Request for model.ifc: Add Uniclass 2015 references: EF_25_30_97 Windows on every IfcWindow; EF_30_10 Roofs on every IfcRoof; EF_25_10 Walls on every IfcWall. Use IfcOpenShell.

First a look at what the model holds.

```python
import ifcopenshell

model = ifcopenshell.open("model.ifc")
print(model.schema)
print("classifications:", [c.Name for c in model.by_type("IfcClassification")])
for ifc_class in ("IfcDoor", "IfcRoof", "IfcStair", "IfcWall", "IfcWindow"):
    print(ifc_class, len(model.by_type(ifc_class)))
```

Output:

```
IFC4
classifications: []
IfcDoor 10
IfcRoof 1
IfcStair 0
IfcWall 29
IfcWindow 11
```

```python
import ifcopenshell
import ifcopenshell.api.classification

model = ifcopenshell.open("model.ifc")

system = ifcopenshell.api.classification.add_classification(model, classification="Uniclass 2015")

codes = {
    "IfcWindow": ("EF_25_30_97", "Windows"),
    "IfcRoof": ("EF_30_10", "Roofs"),
    "IfcWall": ("EF_25_10", "Walls"),
}
for ifc_class, (code, name) in codes.items():
    products = model.by_type(ifc_class)
    ifcopenshell.api.classification.add_reference(
        model, products=products, classification=system, identification=code, name=name
    )
    print(code, len(products))

model.write("model_rev.ifc")
```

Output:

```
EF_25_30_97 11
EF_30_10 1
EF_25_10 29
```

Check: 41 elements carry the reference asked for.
